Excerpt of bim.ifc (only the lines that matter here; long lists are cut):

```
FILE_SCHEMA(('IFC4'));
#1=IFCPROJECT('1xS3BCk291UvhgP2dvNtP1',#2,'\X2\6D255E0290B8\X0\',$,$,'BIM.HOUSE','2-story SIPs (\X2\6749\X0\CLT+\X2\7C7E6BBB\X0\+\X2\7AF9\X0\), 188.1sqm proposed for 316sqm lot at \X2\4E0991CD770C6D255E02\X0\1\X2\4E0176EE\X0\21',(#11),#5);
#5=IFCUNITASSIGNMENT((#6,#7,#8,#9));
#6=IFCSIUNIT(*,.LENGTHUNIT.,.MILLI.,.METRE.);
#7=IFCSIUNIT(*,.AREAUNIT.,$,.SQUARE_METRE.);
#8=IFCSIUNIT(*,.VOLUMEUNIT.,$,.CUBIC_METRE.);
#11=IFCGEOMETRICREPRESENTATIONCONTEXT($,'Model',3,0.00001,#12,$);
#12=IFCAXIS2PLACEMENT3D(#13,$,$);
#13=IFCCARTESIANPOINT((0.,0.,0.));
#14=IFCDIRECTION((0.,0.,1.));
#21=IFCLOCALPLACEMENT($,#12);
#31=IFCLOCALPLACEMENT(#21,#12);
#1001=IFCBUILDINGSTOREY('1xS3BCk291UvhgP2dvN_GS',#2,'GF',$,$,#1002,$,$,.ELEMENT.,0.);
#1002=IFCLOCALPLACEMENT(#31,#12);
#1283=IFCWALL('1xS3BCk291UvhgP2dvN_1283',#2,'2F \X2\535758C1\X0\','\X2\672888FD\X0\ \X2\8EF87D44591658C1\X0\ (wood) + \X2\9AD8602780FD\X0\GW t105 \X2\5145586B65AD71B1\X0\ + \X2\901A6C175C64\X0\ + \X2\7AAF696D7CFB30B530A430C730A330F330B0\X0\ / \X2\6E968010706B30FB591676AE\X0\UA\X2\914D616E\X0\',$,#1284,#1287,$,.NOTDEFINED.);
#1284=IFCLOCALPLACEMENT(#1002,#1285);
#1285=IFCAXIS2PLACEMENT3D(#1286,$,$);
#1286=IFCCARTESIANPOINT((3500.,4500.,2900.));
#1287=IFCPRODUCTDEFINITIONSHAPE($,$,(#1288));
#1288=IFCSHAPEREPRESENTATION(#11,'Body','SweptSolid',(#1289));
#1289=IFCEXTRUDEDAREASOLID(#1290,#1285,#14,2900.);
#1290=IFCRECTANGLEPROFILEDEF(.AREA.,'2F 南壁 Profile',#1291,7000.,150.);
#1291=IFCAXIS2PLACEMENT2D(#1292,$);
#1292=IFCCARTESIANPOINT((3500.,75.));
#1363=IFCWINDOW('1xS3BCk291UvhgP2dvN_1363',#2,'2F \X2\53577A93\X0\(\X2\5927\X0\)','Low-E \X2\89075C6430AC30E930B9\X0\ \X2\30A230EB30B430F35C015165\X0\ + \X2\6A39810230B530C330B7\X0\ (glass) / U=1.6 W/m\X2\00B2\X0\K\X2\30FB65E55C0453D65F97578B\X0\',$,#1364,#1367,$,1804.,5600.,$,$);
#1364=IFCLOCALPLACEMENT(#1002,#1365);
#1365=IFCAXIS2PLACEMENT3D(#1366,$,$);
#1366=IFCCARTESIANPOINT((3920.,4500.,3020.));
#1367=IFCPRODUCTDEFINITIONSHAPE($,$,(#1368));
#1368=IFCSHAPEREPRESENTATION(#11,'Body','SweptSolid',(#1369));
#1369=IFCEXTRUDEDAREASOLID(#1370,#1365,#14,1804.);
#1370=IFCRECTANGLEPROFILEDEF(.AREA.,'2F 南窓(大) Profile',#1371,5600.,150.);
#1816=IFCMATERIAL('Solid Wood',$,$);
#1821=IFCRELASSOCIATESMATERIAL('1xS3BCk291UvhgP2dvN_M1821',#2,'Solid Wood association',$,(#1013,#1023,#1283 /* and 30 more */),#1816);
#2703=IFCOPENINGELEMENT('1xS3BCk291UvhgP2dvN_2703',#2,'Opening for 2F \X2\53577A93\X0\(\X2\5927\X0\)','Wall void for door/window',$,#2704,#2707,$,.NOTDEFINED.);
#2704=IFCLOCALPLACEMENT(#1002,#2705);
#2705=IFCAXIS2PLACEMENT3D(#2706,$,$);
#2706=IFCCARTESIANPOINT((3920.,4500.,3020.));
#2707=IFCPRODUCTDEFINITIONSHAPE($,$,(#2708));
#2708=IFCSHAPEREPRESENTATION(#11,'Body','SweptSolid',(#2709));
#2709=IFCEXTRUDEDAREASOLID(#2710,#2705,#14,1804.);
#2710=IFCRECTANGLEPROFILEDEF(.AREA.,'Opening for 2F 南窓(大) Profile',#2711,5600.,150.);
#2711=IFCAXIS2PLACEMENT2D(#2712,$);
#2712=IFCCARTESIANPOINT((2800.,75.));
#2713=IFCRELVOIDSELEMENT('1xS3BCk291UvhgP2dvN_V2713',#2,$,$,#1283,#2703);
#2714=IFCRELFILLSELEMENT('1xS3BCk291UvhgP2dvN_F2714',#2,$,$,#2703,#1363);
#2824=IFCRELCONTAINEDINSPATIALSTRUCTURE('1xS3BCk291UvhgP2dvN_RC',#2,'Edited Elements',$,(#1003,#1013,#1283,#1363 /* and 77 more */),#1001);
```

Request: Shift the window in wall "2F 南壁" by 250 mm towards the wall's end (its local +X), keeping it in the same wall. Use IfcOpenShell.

```python
import ifcopenshell
import ifcopenshell.api.geometry
import ifcopenshell.util.placement

model = ifcopenshell.open("bim.ifc")

window = model.by_guid("1xS3BCk291UvhgP2dvN_1363")
opening = window.FillsVoids[0].RelatingOpeningElement
wall = opening.VoidsElements[0].RelatingBuildingElement

wall_matrix = ifcopenshell.util.placement.get_local_placement(wall.ObjectPlacement)
shift = wall_matrix[:3, 0] * 250.0
before = ifcopenshell.util.placement.get_local_placement(window.ObjectPlacement)[:3, 3].copy()

# The window is not placed relative to its opening, so move both.
for product in (opening, window):
    matrix = ifcopenshell.util.placement.get_local_placement(product.ObjectPlacement)
    matrix[:3, 3] += shift
    ifcopenshell.api.geometry.edit_object_placement(model, product=product, matrix=matrix, is_si=False)

after = ifcopenshell.util.placement.get_local_placement(window.ObjectPlacement)[:3, 3]
print("window moved by", (after - before).round(3) + 0.0)

model.write("bim-out.ifc")
```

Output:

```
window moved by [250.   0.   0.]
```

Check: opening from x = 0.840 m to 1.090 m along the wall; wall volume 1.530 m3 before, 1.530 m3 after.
